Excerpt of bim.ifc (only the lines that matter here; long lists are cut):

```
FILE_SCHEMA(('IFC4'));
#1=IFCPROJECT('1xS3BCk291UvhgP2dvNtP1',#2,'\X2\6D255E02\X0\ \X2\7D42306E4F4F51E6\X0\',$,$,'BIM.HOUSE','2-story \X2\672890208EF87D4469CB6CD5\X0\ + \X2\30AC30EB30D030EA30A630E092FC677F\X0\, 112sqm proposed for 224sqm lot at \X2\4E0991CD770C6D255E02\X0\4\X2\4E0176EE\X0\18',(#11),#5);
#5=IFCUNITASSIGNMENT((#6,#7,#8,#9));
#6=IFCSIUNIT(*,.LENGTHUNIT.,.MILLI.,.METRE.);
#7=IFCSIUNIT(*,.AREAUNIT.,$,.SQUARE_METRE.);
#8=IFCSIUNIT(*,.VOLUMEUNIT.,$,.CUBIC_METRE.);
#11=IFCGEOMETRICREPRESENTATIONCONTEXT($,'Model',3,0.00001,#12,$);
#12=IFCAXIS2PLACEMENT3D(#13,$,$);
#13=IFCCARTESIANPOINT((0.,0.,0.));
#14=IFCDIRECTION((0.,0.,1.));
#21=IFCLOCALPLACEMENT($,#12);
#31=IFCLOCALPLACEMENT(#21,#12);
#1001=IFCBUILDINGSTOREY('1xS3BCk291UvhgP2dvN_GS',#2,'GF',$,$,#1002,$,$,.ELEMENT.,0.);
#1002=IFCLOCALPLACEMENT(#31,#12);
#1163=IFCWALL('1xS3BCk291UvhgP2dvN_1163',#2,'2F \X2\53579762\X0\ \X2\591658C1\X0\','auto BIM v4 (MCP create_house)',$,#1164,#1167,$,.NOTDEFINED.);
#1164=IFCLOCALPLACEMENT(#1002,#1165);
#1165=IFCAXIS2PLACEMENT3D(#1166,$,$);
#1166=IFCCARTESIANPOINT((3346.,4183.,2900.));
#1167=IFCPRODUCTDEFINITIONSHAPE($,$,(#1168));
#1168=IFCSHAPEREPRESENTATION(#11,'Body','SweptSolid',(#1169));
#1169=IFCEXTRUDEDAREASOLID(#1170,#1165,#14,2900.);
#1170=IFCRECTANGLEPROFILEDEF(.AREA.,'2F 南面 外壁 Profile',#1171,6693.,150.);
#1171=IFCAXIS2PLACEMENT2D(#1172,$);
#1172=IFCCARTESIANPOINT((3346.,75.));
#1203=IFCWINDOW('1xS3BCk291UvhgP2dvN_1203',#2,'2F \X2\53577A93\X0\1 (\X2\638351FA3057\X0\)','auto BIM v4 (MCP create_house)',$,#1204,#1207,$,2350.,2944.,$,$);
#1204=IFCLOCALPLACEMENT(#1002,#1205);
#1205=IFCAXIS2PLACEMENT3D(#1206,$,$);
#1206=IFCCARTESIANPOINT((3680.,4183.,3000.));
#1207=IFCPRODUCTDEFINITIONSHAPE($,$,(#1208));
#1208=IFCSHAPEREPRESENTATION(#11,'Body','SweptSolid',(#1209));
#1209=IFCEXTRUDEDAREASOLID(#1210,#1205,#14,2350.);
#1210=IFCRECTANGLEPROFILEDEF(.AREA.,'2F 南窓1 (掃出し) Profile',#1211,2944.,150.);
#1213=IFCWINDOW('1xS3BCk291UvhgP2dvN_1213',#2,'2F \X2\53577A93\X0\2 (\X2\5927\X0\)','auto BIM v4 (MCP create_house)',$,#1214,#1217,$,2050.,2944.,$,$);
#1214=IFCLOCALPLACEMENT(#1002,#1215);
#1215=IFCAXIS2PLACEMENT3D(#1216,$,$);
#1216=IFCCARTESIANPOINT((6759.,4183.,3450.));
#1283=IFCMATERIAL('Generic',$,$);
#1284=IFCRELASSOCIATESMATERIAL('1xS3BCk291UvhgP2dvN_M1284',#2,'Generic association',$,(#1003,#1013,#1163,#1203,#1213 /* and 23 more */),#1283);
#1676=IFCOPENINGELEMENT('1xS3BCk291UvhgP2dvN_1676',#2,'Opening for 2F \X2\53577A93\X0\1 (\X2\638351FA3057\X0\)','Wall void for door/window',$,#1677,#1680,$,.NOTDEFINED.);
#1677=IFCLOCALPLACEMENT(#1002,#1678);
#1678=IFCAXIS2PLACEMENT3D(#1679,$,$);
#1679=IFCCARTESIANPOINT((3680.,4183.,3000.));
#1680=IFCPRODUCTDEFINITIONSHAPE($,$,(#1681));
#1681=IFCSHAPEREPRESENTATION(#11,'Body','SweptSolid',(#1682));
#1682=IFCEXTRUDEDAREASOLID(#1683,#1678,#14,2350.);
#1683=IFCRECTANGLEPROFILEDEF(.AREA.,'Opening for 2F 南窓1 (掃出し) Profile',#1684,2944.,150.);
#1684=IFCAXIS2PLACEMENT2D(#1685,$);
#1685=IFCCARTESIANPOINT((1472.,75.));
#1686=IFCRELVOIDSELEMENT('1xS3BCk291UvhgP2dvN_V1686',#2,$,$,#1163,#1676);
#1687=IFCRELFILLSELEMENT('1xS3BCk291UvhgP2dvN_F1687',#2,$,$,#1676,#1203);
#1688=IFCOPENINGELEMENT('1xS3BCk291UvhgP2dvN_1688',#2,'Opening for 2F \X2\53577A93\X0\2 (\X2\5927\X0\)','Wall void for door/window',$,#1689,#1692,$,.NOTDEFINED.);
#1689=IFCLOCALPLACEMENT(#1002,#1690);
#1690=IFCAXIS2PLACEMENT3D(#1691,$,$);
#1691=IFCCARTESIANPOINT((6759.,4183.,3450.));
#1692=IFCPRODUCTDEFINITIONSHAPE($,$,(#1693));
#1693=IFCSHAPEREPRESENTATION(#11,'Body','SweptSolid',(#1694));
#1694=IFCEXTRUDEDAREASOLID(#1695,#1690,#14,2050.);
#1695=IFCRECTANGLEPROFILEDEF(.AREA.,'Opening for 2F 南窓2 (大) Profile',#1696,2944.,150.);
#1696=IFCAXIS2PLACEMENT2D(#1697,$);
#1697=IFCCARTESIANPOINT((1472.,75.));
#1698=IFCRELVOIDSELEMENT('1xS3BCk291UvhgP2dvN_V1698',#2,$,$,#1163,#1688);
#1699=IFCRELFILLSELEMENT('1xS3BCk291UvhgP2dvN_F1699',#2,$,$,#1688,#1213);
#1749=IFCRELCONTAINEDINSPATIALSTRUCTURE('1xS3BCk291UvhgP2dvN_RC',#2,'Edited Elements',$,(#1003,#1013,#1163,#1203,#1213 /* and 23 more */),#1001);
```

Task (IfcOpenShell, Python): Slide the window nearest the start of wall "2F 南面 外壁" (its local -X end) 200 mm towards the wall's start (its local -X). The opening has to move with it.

```python
import ifcopenshell
import ifcopenshell.api.geometry
import ifcopenshell.util.placement

model = ifcopenshell.open("bim.ifc")

window = model.by_id(1203)
opening = window.FillsVoids[0].RelatingOpeningElement
wall = opening.VoidsElements[0].RelatingBuildingElement

wall_matrix = ifcopenshell.util.placement.get_local_placement(wall.ObjectPlacement)
shift = wall_matrix[:3, 0] * -200.0
before = ifcopenshell.util.placement.get_local_placement(window.ObjectPlacement)[:3, 3].copy()

# The window is not placed relative to its opening, so move both.
for product in (opening, window):
    matrix = ifcopenshell.util.placement.get_local_placement(product.ObjectPlacement)
    matrix[:3, 3] += shift
    ifcopenshell.api.geometry.edit_object_placement(model, product=product, matrix=matrix, is_si=False)

after = ifcopenshell.util.placement.get_local_placement(window.ObjectPlacement)[:3, 3]
print("window moved by", (after - before).round(3) + 0.0)

model.write("bim_rev.ifc")
```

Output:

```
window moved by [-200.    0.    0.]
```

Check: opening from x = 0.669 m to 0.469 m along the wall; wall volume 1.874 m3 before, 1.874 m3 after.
